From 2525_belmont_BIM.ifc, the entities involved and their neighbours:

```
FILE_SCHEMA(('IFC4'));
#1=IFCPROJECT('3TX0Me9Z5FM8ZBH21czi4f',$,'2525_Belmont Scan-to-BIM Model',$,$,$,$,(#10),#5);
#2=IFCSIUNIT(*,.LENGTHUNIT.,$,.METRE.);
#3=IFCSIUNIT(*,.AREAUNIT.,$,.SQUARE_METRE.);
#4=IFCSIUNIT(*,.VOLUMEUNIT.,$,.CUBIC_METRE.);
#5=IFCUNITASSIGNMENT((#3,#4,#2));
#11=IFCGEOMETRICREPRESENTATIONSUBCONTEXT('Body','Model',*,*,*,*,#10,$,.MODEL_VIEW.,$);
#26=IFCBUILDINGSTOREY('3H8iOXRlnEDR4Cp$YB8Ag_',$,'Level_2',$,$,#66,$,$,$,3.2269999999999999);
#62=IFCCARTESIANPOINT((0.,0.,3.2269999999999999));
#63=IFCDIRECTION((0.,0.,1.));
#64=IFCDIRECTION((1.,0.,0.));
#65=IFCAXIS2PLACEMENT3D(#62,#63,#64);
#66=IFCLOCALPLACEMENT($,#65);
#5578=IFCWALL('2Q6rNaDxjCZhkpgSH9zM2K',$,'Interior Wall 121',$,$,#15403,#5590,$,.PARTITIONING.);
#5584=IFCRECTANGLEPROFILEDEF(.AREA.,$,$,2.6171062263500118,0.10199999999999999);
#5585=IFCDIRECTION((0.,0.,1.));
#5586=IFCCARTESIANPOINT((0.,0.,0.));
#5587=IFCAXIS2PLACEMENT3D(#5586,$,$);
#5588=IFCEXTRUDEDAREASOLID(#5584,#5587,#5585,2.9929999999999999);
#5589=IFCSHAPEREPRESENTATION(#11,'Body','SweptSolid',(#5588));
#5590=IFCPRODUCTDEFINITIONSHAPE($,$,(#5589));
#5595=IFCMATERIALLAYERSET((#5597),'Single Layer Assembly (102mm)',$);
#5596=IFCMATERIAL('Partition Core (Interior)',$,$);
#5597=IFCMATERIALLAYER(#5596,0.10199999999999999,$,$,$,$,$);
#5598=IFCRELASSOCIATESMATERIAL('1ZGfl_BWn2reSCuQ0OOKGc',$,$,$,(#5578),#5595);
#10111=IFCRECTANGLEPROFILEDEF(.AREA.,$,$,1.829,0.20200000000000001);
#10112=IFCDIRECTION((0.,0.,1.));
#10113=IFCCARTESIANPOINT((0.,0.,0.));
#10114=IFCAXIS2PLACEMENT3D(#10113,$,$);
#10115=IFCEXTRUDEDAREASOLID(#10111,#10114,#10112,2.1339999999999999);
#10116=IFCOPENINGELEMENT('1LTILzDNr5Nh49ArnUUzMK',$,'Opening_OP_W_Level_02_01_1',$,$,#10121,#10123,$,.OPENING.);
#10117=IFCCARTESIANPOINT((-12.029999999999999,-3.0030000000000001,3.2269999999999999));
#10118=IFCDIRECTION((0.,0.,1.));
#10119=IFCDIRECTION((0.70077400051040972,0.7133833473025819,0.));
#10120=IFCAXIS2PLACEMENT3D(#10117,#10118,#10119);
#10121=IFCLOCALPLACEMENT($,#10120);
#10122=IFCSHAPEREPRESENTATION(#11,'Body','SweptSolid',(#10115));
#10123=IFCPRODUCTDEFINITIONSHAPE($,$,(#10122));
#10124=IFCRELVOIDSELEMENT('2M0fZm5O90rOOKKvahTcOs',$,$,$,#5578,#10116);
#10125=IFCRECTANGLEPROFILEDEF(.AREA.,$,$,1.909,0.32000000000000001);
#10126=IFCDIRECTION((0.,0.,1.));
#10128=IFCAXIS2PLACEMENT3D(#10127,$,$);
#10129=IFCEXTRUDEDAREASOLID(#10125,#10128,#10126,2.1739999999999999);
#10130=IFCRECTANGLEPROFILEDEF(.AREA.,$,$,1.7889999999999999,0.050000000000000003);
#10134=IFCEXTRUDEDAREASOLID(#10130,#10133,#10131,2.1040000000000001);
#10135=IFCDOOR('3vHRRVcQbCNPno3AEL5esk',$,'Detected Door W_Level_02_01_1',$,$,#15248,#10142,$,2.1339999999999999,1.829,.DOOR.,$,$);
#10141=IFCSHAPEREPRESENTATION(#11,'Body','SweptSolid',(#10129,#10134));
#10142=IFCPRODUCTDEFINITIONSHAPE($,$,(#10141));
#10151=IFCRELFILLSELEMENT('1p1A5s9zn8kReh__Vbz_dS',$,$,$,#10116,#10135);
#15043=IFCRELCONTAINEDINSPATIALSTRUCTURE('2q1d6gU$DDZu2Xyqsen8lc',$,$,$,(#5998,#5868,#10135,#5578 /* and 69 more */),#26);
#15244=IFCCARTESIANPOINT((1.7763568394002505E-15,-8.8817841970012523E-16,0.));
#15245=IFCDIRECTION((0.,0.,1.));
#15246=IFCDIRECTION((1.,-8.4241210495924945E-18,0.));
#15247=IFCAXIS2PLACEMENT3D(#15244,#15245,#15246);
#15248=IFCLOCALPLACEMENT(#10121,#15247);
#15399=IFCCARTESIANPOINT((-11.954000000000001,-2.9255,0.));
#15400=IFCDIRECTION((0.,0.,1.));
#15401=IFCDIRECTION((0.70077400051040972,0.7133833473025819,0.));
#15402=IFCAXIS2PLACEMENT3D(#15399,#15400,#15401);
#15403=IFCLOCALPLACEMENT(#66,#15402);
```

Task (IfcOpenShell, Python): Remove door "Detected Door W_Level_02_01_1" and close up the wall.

```python
import ifcopenshell
import ifcopenshell.api.feature
import ifcopenshell.api.root
import ifcopenshell.geom
import ifcopenshell.util.shape

model = ifcopenshell.open("2525_belmont_BIM.ifc")
settings = ifcopenshell.geom.settings()


def volume(element):
    """Net volume in cubic metres, openings subtracted."""
    shape = ifcopenshell.geom.create_shape(settings, element)
    return ifcopenshell.util.shape.get_volume(shape.geometry)


door = model.by_guid("3vHRRVcQbCNPno3AEL5esk")
opening = door.FillsVoids[0].RelatingOpeningElement
wall = opening.VoidsElements[0].RelatingBuildingElement
before = volume(wall)

ifcopenshell.api.root.remove_product(model, product=door)
ifcopenshell.api.feature.remove_feature(model, feature=opening)

after = volume(wall)

print(f"wall volume {before:.3f} -> {after:.3f} m3")

model.write("2525_belmont_BIM_updated.ifc")
```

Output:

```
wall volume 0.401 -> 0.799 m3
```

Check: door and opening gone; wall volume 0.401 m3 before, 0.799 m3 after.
